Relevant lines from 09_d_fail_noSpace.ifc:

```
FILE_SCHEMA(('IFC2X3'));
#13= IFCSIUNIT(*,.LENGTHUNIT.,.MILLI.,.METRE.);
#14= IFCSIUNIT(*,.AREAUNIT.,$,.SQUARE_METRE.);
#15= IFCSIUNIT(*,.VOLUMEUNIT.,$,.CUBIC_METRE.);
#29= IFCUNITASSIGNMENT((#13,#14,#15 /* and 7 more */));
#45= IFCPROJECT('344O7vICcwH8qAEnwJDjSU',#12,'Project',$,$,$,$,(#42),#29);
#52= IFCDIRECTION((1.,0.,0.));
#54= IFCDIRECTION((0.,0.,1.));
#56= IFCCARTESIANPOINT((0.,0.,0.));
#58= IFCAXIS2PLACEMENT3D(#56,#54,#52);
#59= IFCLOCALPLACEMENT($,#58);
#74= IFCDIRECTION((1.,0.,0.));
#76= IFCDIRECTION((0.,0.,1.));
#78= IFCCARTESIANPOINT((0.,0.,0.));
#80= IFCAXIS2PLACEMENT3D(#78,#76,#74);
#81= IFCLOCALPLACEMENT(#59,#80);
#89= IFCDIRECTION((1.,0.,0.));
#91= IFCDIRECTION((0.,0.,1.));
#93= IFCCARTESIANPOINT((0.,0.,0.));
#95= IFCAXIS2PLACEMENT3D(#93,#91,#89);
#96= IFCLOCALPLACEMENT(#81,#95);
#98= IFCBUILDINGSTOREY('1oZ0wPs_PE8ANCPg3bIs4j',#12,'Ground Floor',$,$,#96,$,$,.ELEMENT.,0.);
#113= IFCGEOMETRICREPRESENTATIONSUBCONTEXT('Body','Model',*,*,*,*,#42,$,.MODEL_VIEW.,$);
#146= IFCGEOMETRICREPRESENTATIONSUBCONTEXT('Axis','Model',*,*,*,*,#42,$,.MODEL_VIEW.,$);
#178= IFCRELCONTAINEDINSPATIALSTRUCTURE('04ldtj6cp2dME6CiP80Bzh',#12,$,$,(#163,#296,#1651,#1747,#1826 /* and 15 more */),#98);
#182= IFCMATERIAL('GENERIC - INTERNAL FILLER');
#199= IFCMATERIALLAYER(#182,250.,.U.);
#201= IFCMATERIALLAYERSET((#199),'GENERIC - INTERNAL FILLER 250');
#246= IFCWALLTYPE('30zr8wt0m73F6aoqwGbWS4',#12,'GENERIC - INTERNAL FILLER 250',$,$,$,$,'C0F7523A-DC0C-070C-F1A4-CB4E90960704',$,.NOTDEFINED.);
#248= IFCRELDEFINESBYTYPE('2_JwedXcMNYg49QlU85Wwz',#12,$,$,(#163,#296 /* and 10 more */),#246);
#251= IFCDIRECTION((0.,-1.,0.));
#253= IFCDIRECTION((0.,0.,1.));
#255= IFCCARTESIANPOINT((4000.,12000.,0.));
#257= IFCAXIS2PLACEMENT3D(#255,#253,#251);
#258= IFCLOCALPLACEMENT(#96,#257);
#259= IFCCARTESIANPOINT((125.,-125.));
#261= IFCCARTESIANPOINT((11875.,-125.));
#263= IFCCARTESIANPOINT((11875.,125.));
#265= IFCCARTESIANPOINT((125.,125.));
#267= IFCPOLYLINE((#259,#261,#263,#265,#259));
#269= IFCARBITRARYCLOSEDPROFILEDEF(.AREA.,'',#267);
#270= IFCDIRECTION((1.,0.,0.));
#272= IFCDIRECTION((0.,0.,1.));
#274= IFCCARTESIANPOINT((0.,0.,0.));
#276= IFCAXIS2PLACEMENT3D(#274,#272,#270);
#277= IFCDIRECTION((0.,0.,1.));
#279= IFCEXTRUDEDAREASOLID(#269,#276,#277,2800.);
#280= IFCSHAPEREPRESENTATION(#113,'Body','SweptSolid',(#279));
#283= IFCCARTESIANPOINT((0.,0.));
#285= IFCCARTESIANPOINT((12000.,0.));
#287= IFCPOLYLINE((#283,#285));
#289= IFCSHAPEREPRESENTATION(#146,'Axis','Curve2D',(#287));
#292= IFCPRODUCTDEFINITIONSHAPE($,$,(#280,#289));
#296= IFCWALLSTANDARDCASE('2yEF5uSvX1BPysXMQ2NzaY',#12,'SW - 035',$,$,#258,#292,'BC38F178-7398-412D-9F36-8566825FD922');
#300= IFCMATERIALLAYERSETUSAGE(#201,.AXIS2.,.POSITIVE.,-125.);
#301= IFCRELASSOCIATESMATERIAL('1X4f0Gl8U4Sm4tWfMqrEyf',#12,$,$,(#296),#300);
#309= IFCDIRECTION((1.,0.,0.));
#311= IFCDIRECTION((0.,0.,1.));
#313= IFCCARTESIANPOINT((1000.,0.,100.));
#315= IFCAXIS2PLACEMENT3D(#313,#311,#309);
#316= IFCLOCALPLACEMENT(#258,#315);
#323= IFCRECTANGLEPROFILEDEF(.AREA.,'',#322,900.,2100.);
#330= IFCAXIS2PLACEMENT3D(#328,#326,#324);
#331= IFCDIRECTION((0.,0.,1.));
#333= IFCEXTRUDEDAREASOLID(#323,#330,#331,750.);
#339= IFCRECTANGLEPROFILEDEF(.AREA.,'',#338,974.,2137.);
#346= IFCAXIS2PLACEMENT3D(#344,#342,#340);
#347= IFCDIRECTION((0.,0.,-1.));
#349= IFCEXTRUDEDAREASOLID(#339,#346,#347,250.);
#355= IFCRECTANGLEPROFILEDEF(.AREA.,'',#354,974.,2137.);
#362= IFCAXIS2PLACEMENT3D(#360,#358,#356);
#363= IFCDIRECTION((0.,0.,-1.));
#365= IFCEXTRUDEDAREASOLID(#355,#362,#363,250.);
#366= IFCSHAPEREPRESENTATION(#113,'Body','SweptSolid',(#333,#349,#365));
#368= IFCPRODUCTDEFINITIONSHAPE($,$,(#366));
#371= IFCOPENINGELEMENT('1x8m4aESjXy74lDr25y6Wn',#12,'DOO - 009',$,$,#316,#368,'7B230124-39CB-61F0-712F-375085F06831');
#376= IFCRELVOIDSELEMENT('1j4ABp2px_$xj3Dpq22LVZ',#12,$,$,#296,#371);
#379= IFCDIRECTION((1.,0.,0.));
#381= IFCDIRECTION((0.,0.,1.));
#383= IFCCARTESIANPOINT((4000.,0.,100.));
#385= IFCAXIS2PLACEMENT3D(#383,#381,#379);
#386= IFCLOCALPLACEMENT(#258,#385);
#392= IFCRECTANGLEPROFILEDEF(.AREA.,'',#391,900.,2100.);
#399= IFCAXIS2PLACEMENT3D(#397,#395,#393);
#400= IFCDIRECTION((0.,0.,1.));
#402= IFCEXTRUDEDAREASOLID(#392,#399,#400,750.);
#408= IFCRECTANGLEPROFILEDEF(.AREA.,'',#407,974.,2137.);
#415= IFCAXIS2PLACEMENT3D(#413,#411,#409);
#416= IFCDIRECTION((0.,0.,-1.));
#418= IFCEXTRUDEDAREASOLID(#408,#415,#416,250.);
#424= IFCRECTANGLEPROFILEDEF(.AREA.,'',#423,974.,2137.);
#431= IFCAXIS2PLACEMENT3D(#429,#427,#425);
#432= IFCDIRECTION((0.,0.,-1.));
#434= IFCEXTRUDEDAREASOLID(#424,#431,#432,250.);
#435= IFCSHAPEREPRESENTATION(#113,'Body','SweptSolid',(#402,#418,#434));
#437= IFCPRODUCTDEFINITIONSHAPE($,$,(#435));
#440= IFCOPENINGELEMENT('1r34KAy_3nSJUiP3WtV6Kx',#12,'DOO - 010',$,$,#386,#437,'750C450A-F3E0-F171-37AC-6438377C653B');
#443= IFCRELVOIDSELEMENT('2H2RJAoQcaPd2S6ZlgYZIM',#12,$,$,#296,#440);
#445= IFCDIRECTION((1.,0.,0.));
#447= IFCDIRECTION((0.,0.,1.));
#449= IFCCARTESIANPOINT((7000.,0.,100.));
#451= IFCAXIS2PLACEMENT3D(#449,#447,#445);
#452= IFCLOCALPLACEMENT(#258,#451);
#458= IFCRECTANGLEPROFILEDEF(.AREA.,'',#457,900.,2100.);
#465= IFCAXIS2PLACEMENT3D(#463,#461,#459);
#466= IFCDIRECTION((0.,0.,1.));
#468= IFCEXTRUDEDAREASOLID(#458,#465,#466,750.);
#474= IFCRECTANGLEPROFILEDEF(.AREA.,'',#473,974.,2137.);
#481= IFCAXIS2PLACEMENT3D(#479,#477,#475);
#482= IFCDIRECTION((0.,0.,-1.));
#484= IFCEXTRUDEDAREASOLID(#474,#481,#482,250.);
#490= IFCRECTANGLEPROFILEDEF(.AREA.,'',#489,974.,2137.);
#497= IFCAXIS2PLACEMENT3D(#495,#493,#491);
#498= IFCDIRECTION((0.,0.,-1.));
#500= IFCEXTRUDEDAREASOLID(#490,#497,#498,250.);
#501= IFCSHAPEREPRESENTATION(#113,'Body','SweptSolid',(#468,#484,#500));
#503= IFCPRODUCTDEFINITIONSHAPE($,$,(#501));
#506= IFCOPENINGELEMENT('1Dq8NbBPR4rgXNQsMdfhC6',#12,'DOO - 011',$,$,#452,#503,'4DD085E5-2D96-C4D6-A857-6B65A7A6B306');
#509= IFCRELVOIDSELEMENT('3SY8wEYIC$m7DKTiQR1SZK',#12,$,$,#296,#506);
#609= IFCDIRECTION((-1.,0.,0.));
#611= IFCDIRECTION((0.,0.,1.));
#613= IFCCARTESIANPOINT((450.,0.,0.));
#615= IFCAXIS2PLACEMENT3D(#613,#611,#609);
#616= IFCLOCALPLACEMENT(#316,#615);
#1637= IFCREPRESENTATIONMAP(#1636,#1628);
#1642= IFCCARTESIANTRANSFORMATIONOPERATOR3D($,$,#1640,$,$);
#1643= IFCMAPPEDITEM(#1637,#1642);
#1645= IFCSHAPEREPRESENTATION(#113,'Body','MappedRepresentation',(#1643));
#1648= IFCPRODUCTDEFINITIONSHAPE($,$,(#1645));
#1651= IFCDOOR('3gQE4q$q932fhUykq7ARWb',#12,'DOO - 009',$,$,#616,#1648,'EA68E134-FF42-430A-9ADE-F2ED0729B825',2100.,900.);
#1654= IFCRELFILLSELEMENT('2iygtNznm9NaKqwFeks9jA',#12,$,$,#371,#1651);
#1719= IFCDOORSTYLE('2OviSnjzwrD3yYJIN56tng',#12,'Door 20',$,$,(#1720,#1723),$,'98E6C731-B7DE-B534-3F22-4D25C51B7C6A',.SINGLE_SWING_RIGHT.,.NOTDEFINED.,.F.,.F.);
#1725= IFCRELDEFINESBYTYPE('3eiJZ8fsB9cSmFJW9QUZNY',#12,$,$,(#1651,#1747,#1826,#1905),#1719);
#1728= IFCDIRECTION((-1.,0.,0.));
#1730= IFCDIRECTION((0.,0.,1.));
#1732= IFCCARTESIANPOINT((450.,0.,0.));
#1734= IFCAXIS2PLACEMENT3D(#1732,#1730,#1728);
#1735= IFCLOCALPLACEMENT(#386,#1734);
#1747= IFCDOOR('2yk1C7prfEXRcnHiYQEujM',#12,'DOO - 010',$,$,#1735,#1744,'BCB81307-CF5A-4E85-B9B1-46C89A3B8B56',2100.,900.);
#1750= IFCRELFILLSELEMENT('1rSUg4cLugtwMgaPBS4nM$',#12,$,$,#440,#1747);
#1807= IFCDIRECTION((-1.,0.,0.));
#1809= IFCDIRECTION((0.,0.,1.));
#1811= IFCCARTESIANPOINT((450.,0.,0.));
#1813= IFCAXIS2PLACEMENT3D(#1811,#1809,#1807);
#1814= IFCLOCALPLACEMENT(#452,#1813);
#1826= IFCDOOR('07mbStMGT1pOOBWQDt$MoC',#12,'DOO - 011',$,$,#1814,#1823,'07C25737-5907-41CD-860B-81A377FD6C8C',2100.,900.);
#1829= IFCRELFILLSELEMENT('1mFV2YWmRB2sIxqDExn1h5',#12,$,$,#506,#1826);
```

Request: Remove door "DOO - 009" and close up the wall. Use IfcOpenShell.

```python
import ifcopenshell
import ifcopenshell.api.feature
import ifcopenshell.api.root
import ifcopenshell.geom
import ifcopenshell.util.shape

model = ifcopenshell.open("09_d_fail_noSpace.ifc")
settings = ifcopenshell.geom.settings()


def volume(element):
    """Net volume in cubic metres, openings subtracted."""
    shape = ifcopenshell.geom.create_shape(settings, element)
    return ifcopenshell.util.shape.get_volume(shape.geometry)


door = model.by_guid("3gQE4q$q932fhUykq7ARWb")
opening = door.FillsVoids[0].RelatingOpeningElement
wall = opening.VoidsElements[0].RelatingBuildingElement
before = volume(wall)

ifcopenshell.api.root.remove_product(model, product=door)
ifcopenshell.api.feature.remove_feature(model, feature=opening)

after = volume(wall)

print(f"wall volume {before:.3f} -> {after:.3f} m3")

model.write("09_d_fail_noSpace_v2.ifc")
```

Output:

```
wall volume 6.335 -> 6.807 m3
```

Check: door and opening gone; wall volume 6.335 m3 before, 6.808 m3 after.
